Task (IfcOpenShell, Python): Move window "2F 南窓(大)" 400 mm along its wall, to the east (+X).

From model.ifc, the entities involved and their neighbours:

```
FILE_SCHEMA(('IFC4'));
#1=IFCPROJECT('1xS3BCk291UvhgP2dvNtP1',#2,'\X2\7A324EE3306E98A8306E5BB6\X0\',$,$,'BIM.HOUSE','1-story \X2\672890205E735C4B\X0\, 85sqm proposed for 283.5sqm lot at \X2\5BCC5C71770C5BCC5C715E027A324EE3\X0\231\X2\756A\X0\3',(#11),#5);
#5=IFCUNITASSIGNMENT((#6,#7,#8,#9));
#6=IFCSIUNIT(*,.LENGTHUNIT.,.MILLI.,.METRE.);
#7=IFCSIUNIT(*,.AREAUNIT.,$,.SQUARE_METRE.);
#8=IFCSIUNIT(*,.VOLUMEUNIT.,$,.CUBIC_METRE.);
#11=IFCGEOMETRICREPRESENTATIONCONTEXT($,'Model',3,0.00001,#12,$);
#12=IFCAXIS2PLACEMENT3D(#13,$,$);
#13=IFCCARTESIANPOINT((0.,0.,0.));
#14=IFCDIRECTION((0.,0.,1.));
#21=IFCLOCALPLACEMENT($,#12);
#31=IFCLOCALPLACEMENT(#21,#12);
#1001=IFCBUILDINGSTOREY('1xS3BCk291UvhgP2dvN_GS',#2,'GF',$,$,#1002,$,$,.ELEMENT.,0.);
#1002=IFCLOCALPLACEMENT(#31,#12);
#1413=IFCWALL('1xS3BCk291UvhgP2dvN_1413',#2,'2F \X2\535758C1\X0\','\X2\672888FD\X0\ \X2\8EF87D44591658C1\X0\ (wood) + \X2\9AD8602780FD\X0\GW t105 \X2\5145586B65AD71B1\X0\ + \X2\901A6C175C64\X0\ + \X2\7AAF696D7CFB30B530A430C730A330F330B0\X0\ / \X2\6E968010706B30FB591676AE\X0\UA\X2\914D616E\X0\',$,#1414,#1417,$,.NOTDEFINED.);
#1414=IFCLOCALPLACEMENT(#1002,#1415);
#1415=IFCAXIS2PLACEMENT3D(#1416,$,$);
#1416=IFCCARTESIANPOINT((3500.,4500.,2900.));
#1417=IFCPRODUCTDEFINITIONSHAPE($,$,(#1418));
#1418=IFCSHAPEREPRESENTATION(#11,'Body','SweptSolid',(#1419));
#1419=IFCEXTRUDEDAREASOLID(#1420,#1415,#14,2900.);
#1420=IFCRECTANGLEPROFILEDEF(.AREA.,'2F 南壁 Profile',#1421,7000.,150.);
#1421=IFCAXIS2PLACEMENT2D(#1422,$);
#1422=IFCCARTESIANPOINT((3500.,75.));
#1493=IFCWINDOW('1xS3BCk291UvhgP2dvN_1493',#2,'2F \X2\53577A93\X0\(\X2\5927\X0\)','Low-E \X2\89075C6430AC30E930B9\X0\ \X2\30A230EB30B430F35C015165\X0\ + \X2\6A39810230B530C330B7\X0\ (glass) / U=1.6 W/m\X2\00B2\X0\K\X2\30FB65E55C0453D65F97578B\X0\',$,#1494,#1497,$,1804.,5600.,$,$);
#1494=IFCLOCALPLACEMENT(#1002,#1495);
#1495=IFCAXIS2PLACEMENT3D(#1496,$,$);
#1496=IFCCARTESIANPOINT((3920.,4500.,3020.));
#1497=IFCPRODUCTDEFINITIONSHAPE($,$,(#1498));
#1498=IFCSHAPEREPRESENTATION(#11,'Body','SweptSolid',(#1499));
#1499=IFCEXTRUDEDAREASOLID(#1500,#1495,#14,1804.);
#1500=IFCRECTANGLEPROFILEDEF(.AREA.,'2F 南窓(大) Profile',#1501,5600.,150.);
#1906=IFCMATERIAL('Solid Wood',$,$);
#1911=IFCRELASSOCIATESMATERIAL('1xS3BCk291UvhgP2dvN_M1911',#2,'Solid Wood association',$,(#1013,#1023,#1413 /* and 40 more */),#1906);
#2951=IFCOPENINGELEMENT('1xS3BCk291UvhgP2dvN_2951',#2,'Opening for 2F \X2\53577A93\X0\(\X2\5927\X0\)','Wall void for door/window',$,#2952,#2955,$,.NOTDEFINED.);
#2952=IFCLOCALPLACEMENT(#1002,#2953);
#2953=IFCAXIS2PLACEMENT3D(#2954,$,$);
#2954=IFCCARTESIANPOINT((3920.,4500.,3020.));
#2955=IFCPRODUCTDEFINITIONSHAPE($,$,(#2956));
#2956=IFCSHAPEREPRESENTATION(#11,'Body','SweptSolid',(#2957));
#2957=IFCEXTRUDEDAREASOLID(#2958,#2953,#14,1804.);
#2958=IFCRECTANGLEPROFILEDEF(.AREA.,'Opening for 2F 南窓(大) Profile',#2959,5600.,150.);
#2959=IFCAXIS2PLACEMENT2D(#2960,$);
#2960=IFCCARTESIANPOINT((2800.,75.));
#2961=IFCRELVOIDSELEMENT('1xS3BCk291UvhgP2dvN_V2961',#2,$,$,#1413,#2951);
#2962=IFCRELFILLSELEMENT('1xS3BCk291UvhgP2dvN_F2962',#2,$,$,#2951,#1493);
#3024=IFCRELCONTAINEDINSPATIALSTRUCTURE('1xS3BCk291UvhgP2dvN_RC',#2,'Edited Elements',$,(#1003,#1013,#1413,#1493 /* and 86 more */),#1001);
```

```python
import ifcopenshell
import ifcopenshell.api.geometry
import ifcopenshell.util.placement
import ifcopenshell.util.unit

model = ifcopenshell.open("model.ifc")
unit_scale = ifcopenshell.util.unit.calculate_unit_scale(model)

window = model.by_id(1493)
opening = window.FillsVoids[0].RelatingOpeningElement
wall = opening.VoidsElements[0].RelatingBuildingElement

wall_matrix = ifcopenshell.util.placement.get_local_placement(wall.ObjectPlacement)
shift = wall_matrix[:3, 0] * 0.4 / unit_scale
before = ifcopenshell.util.placement.get_local_placement(window.ObjectPlacement)[:3, 3].copy()

# The window is not placed relative to its opening, so move both.
for product in (opening, window):
    matrix = ifcopenshell.util.placement.get_local_placement(product.ObjectPlacement)
    matrix[:3, 3] += shift
    ifcopenshell.api.geometry.edit_object_placement(model, product=product, matrix=matrix, is_si=False)

after = ifcopenshell.util.placement.get_local_placement(window.ObjectPlacement)[:3, 3]
print("window moved by", (after - before).round(3) + 0.0)

model.write("model-out.ifc")
```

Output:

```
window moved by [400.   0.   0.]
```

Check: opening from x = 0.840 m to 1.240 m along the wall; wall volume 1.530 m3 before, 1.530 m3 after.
